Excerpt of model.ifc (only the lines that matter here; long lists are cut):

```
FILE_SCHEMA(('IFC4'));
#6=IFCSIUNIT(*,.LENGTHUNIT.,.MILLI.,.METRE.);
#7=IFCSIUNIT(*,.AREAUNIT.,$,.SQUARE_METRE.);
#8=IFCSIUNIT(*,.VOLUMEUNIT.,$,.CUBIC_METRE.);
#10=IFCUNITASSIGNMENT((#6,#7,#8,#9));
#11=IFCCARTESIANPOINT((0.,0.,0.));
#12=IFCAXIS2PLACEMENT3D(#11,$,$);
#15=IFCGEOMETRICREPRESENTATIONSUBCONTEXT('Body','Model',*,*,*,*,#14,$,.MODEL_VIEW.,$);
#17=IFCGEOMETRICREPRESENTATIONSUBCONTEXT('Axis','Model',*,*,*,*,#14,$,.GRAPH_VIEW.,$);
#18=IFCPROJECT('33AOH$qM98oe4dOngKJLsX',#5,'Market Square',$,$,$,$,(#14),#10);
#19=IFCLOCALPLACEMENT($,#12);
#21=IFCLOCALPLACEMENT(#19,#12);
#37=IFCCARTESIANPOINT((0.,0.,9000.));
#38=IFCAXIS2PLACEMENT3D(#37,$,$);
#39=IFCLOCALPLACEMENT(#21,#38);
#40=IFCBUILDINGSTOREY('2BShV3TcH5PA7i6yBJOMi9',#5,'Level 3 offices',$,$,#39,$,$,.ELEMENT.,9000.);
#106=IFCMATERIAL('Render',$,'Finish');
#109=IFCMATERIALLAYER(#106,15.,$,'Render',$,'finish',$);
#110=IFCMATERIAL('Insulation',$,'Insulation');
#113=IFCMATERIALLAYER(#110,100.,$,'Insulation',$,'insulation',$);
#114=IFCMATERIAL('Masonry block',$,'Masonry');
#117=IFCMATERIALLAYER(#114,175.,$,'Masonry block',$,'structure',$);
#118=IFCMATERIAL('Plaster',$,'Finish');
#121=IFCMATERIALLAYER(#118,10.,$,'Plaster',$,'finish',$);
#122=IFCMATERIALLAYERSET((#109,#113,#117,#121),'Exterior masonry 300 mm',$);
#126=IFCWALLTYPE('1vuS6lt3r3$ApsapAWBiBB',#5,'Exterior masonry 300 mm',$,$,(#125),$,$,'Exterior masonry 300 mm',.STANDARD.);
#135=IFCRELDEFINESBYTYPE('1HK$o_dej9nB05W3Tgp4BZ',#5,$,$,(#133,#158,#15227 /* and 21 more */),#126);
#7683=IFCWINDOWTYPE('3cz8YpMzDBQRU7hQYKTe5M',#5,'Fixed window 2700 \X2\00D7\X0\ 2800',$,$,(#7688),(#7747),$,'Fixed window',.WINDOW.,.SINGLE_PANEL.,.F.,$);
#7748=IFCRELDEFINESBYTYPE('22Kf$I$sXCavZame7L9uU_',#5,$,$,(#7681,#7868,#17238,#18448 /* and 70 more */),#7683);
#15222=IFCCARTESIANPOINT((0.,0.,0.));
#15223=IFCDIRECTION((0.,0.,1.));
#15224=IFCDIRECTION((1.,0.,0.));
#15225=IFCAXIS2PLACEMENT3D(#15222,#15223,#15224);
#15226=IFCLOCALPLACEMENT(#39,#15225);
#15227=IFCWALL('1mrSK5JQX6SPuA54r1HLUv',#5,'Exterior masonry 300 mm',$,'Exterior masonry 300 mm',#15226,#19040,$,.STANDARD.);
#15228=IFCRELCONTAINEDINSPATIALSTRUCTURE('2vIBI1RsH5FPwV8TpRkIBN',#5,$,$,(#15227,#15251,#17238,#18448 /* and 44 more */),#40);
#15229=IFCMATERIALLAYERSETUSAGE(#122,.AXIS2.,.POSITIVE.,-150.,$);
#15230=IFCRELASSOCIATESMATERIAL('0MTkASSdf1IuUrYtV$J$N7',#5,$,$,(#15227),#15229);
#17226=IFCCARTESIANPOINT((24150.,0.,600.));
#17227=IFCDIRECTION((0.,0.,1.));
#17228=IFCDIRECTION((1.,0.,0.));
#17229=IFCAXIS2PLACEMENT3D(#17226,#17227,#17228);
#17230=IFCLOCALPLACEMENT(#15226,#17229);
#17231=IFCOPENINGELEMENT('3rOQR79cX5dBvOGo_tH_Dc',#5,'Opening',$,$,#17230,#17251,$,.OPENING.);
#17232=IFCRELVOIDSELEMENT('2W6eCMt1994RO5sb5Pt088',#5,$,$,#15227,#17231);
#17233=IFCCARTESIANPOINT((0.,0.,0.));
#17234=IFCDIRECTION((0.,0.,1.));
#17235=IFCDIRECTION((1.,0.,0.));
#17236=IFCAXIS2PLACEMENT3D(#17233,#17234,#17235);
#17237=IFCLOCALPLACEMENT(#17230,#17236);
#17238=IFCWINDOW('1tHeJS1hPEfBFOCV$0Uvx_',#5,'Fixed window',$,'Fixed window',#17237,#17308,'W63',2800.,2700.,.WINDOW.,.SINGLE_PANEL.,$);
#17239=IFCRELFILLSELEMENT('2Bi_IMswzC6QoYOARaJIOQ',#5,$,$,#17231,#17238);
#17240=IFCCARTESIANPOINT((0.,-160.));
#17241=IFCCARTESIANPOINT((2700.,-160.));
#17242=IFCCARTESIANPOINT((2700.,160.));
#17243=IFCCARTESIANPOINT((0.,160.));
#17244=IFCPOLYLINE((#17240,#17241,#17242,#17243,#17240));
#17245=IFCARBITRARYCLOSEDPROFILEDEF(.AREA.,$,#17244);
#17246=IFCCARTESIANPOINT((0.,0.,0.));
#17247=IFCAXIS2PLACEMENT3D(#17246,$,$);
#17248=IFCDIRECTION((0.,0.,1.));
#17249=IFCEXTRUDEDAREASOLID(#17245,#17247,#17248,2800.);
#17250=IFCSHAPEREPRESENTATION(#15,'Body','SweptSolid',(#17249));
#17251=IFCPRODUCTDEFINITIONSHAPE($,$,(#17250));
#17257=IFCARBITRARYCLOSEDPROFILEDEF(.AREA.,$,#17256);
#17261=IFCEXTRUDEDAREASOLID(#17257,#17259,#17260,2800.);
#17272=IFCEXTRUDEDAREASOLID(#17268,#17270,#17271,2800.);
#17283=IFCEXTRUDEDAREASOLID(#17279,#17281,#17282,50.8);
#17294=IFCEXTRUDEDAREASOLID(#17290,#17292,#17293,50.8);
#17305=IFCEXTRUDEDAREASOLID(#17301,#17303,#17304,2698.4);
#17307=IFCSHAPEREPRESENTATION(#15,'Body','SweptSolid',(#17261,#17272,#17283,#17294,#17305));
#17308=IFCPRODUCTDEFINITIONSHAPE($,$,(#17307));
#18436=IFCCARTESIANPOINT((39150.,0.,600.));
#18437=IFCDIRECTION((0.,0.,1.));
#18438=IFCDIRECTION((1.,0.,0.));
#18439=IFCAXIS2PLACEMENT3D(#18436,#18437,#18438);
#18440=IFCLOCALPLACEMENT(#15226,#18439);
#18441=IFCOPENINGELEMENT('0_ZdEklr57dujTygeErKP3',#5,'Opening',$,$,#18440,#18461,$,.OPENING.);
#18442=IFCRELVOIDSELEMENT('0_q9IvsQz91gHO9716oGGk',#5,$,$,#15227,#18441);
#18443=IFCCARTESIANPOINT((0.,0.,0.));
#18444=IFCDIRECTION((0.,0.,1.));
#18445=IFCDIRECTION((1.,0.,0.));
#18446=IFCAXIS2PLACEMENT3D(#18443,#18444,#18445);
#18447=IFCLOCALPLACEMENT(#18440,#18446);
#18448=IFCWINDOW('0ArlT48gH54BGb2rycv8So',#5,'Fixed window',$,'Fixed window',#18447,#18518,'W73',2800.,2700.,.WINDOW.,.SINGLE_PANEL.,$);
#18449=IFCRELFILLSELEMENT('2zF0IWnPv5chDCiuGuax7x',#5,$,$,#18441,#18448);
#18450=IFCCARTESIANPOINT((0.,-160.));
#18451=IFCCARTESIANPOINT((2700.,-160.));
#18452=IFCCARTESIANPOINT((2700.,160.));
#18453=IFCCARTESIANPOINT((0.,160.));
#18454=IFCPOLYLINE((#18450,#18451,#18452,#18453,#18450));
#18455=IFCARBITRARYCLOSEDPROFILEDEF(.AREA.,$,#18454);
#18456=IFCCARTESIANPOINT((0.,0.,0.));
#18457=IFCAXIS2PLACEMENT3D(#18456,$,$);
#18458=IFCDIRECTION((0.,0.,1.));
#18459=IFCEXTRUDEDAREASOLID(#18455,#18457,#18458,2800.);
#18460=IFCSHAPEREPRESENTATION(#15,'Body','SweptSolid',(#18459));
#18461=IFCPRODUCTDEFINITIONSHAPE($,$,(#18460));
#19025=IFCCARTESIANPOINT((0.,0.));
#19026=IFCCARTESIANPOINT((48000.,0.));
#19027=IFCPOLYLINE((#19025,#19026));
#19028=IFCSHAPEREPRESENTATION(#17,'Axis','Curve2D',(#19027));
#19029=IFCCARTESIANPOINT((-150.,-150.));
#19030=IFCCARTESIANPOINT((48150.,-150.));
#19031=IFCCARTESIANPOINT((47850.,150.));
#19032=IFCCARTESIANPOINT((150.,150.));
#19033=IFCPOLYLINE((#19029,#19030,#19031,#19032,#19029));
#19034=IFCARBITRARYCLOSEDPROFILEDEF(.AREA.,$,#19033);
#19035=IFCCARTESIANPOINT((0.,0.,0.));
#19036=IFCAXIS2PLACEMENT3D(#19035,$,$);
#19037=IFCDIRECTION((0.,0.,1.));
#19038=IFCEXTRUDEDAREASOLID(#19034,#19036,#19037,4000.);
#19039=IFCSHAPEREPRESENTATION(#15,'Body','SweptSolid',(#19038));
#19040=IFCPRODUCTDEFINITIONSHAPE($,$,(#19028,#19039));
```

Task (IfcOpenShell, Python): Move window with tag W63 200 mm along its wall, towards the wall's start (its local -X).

```python
import ifcopenshell
import ifcopenshell.api.geometry
import ifcopenshell.util.placement
import ifcopenshell.util.unit

model = ifcopenshell.open("model.ifc")
unit_scale = ifcopenshell.util.unit.calculate_unit_scale(model)

window = model.by_guid("1tHeJS1hPEfBFOCV$0Uvx_")
opening = window.FillsVoids[0].RelatingOpeningElement
wall = opening.VoidsElements[0].RelatingBuildingElement

wall_matrix = ifcopenshell.util.placement.get_local_placement(wall.ObjectPlacement)
shift = wall_matrix[:3, 0] * -0.2 / unit_scale
before = ifcopenshell.util.placement.get_local_placement(window.ObjectPlacement)[:3, 3].copy()

# The window is placed relative to its opening, so it follows when the opening moves.
matrix = ifcopenshell.util.placement.get_local_placement(opening.ObjectPlacement)
matrix[:3, 3] += shift
ifcopenshell.api.geometry.edit_object_placement(
    model, product=opening, matrix=matrix, is_si=False, should_transform_children=True
)

after = ifcopenshell.util.placement.get_local_placement(window.ObjectPlacement)[:3, 3]
print("window moved by", (after - before).round(3) + 0.0)

model.write("model_rev.ifc")
```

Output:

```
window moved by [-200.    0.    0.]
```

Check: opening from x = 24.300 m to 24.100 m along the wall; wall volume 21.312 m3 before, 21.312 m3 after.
